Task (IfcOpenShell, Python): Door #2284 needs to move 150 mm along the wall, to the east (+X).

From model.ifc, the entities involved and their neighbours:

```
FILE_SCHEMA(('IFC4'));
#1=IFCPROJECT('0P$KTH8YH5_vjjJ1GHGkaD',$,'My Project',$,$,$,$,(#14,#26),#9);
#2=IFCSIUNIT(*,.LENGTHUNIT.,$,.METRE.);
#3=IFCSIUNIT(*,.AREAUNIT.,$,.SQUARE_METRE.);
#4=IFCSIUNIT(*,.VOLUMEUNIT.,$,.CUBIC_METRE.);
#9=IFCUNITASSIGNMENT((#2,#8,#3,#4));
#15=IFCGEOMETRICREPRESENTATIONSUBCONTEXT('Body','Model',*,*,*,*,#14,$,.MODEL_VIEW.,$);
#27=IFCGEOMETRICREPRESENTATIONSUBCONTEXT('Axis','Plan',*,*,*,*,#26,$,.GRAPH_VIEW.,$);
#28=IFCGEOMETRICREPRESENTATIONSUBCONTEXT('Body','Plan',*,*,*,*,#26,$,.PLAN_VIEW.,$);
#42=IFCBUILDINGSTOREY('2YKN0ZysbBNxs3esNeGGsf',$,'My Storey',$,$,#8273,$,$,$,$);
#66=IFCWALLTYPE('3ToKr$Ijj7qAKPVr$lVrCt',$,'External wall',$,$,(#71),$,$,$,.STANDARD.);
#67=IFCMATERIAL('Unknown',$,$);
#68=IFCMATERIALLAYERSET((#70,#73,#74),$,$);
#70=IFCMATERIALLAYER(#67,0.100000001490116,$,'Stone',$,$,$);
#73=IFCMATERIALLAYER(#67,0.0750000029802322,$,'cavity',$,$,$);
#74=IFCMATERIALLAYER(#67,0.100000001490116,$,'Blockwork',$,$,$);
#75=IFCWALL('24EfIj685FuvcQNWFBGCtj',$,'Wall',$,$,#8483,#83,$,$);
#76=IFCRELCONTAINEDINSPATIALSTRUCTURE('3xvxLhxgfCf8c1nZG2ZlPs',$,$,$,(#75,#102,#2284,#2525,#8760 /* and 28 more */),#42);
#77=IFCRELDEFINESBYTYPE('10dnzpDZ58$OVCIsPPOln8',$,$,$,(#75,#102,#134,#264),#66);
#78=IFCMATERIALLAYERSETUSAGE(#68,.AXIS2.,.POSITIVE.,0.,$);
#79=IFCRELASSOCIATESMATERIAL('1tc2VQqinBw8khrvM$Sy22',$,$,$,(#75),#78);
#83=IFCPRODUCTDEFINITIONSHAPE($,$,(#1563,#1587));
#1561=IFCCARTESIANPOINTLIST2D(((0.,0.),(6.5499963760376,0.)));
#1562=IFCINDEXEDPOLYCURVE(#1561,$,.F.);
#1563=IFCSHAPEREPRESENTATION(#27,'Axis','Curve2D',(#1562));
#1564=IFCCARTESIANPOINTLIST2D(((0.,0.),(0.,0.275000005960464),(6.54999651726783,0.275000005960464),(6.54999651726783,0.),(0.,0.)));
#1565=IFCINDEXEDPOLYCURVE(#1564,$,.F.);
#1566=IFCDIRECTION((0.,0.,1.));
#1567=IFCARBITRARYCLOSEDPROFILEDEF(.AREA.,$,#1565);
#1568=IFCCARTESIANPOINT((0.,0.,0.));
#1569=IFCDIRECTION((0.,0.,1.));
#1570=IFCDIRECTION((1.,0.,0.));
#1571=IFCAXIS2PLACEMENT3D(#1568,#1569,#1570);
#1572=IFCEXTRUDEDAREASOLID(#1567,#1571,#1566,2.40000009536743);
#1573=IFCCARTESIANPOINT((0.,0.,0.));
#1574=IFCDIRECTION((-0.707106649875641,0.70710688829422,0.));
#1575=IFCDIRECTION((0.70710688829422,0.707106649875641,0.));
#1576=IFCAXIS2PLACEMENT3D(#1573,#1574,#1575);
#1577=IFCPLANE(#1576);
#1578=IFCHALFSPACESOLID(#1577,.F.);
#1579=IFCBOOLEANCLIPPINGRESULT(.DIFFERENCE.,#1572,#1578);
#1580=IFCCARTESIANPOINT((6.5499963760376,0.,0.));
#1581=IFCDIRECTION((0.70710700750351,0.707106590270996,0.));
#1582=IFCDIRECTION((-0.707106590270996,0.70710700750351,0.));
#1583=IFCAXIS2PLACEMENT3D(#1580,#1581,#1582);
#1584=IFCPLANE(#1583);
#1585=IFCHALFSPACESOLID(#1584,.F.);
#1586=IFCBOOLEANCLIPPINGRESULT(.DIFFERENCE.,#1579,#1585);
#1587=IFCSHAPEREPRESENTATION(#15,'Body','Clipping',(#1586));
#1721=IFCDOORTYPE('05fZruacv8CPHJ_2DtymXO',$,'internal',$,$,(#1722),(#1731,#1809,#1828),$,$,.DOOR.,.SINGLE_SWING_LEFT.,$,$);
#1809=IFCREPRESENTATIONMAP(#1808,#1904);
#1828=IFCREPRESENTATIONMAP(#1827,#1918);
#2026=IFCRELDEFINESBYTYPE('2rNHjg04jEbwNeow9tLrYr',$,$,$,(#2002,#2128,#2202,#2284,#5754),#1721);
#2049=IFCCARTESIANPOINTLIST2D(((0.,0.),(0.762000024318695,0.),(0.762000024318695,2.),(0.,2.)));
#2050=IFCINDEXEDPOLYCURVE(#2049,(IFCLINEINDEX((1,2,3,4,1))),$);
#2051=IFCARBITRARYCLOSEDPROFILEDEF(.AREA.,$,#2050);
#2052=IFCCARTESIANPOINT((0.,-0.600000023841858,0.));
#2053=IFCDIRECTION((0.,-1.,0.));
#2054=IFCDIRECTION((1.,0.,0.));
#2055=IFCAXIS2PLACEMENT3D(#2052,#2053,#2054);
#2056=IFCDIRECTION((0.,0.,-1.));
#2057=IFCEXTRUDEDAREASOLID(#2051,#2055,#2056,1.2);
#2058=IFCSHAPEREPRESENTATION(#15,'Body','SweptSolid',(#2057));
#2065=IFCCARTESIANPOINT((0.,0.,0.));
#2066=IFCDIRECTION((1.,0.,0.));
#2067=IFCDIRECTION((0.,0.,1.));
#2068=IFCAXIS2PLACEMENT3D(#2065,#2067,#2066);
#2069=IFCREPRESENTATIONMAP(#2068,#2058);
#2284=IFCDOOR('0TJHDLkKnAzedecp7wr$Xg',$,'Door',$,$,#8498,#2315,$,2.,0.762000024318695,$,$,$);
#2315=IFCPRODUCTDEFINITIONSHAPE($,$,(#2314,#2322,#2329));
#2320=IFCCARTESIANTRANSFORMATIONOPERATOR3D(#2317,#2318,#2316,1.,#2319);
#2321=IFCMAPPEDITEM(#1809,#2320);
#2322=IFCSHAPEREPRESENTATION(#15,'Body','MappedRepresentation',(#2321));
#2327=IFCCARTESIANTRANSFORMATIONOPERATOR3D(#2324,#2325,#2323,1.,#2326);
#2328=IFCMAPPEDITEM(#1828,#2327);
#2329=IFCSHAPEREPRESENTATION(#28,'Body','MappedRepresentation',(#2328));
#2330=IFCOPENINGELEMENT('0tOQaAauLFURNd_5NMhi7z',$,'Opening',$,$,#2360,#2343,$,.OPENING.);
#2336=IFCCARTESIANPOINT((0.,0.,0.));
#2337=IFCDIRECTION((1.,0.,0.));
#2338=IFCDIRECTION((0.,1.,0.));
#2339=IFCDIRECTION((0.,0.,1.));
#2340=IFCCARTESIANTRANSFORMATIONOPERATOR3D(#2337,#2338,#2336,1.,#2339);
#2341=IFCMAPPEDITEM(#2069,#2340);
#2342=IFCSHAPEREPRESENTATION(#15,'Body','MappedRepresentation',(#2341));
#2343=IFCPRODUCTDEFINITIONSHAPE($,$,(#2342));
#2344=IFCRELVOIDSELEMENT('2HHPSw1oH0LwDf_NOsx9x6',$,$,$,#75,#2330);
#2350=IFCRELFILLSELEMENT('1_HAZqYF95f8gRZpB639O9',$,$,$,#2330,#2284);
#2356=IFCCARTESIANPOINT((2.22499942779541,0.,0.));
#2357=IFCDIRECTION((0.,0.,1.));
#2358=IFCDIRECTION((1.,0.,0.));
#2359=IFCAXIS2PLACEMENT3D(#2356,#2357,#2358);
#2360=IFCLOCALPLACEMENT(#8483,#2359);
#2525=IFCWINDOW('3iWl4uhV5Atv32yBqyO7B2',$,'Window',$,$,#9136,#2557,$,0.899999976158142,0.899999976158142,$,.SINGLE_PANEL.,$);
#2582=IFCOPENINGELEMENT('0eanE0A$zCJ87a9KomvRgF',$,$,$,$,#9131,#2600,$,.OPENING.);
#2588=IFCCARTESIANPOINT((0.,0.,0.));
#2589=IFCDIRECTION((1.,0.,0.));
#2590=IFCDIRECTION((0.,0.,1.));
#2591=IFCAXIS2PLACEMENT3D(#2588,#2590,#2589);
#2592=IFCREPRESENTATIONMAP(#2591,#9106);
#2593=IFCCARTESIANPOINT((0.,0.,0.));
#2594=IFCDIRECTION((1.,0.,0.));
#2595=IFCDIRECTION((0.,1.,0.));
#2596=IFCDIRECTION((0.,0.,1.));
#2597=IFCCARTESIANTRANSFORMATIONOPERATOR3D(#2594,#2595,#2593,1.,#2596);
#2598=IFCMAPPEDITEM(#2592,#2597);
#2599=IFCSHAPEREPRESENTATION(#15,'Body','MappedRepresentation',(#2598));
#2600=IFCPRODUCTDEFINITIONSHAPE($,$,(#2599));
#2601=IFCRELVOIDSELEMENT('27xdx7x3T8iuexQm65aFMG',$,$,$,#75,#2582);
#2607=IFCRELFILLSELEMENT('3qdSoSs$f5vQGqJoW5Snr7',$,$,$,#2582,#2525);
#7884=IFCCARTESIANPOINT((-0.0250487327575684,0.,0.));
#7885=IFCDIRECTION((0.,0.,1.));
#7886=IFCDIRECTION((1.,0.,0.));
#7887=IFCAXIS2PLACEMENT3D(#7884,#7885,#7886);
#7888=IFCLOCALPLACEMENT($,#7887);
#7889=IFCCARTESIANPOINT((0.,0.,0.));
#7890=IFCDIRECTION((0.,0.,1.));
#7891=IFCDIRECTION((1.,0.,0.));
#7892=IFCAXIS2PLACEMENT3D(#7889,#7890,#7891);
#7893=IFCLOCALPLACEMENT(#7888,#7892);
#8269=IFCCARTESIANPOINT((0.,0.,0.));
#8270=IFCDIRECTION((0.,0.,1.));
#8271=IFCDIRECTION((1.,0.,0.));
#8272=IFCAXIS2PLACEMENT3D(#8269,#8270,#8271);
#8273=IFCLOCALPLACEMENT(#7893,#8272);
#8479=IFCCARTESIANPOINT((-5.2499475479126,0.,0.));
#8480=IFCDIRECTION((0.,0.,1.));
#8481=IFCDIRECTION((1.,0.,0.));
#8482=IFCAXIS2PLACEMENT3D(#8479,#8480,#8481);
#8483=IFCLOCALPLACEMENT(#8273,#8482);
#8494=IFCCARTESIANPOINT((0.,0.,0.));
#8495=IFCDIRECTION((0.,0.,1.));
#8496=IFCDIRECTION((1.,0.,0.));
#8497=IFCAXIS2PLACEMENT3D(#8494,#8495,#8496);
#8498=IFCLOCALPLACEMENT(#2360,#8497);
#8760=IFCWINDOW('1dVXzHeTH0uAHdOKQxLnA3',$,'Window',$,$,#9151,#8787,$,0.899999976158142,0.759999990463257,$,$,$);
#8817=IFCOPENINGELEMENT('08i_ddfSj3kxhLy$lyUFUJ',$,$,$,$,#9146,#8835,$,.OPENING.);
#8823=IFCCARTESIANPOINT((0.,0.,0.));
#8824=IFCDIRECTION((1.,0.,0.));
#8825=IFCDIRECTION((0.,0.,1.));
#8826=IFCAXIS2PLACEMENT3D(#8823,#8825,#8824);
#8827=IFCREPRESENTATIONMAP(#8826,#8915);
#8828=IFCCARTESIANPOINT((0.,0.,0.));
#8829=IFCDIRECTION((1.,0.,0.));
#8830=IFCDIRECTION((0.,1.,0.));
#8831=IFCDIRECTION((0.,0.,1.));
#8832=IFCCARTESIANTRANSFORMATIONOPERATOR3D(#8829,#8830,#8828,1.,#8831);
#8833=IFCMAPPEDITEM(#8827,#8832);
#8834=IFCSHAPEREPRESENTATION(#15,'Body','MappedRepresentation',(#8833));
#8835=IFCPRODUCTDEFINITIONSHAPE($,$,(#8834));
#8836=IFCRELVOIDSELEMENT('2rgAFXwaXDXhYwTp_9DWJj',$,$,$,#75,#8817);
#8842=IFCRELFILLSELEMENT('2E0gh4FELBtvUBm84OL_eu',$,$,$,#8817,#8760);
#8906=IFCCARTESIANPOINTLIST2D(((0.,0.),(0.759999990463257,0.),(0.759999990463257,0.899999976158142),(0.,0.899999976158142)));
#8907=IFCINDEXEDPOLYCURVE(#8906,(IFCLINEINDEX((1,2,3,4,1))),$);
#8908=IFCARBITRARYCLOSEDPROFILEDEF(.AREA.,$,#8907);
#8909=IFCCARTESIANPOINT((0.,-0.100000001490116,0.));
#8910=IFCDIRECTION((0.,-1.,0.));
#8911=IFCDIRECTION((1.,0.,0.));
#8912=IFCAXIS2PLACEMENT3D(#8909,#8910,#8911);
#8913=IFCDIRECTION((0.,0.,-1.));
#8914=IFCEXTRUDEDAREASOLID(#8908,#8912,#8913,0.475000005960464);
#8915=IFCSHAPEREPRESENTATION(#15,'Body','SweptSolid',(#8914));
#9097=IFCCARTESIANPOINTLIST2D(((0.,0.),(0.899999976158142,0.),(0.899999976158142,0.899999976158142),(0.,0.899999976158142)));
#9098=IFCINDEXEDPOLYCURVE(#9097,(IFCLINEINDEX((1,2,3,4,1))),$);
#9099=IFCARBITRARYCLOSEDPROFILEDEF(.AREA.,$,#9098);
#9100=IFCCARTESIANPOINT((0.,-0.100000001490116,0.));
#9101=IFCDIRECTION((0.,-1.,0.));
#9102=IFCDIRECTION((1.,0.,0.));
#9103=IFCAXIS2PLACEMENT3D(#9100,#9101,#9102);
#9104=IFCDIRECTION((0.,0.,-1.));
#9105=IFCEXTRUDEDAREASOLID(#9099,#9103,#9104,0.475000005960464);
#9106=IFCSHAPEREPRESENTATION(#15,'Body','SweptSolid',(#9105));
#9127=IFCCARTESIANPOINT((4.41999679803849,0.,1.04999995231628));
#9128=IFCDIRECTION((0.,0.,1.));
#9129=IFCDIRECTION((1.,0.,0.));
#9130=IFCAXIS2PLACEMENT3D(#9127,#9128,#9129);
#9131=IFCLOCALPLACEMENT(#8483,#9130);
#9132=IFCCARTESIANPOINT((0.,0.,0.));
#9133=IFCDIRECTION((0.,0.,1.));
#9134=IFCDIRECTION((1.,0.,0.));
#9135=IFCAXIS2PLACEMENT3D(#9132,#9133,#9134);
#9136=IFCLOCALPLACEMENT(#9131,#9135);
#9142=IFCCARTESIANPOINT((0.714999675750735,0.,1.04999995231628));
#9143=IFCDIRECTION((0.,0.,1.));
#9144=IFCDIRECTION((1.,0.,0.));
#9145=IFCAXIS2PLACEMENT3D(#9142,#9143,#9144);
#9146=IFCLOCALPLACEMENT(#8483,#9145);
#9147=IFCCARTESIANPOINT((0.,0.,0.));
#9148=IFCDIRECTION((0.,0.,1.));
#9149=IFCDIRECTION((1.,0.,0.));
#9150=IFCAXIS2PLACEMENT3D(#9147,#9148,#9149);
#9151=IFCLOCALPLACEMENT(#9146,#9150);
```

```python
import ifcopenshell
import ifcopenshell.api.geometry
import ifcopenshell.util.placement
import ifcopenshell.util.unit

model = ifcopenshell.open("model.ifc")
unit_scale = ifcopenshell.util.unit.calculate_unit_scale(model)

door = model.by_guid("0TJHDLkKnAzedecp7wr$Xg")
opening = door.FillsVoids[0].RelatingOpeningElement
wall = opening.VoidsElements[0].RelatingBuildingElement

wall_matrix = ifcopenshell.util.placement.get_local_placement(wall.ObjectPlacement)
shift = wall_matrix[:3, 0] * 0.15 / unit_scale
before = ifcopenshell.util.placement.get_local_placement(door.ObjectPlacement)[:3, 3].copy()

# The door is placed relative to its opening, so it follows when the opening moves.
matrix = ifcopenshell.util.placement.get_local_placement(opening.ObjectPlacement)
matrix[:3, 3] += shift
ifcopenshell.api.geometry.edit_object_placement(
    model, product=opening, matrix=matrix, is_si=False, should_transform_children=True
)

after = ifcopenshell.util.placement.get_local_placement(door.ObjectPlacement)[:3, 3]
print("door moved by", (after - before).round(3) + 0.0)

model.write("model_rev.ifc")
```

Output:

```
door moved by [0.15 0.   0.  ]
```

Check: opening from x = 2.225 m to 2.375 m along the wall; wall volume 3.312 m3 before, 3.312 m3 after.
